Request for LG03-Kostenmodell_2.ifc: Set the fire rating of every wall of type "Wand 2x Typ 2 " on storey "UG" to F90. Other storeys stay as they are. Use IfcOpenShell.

First a look at what the model holds.

```python
import ifcopenshell
import ifcopenshell.util.element

model = ifcopenshell.open("LG03-Kostenmodell_2.ifc")
print(model.schema)
storey = next(s for s in model.by_type("IfcBuildingStorey") if s.Name == "UG")
walls = [e for e in ifcopenshell.util.element.get_decomposition(storey) if e.is_a("IfcWall")]
seen = {}
for e in walls:
    element_type = ifcopenshell.util.element.get_type(e)
    key = (element_type.Name if element_type != e and element_type else None, ifcopenshell.util.element.get_pset(e, "Pset_WallCommon", "FireRating"))
    seen[key] = seen.get(key, 0) + 1
for (name, value), count in sorted(seen.items(), key=str):
    print(count, "x", name, "|", value)
```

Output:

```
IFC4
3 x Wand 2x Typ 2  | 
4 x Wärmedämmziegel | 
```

```python
import ifcopenshell
import ifcopenshell.api.pset
import ifcopenshell.util.element

model = ifcopenshell.open("LG03-Kostenmodell_2.ifc")

storey = next(s for s in model.by_type("IfcBuildingStorey") if s.Name == "UG")
walls = [e for e in ifcopenshell.util.element.get_decomposition(storey) if e.is_a("IfcWall")]

count = 0
for e in walls:
    element_type = ifcopenshell.util.element.get_type(e)
    if element_type in (None, e) or element_type.Name != "Wand 2x Typ 2 ":
        continue
    # add_pset returns the element's existing set when there is one.
    pset = ifcopenshell.api.pset.add_pset(model, product=e, name="Pset_WallCommon")
    ifcopenshell.api.pset.edit_pset(model, pset=pset, properties={"FireRating": "F90"})
    count += 1

print(count, "walls updated")

model.write("LG03-Kostenmodell_2_rev.ifc")
```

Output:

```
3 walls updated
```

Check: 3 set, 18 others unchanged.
